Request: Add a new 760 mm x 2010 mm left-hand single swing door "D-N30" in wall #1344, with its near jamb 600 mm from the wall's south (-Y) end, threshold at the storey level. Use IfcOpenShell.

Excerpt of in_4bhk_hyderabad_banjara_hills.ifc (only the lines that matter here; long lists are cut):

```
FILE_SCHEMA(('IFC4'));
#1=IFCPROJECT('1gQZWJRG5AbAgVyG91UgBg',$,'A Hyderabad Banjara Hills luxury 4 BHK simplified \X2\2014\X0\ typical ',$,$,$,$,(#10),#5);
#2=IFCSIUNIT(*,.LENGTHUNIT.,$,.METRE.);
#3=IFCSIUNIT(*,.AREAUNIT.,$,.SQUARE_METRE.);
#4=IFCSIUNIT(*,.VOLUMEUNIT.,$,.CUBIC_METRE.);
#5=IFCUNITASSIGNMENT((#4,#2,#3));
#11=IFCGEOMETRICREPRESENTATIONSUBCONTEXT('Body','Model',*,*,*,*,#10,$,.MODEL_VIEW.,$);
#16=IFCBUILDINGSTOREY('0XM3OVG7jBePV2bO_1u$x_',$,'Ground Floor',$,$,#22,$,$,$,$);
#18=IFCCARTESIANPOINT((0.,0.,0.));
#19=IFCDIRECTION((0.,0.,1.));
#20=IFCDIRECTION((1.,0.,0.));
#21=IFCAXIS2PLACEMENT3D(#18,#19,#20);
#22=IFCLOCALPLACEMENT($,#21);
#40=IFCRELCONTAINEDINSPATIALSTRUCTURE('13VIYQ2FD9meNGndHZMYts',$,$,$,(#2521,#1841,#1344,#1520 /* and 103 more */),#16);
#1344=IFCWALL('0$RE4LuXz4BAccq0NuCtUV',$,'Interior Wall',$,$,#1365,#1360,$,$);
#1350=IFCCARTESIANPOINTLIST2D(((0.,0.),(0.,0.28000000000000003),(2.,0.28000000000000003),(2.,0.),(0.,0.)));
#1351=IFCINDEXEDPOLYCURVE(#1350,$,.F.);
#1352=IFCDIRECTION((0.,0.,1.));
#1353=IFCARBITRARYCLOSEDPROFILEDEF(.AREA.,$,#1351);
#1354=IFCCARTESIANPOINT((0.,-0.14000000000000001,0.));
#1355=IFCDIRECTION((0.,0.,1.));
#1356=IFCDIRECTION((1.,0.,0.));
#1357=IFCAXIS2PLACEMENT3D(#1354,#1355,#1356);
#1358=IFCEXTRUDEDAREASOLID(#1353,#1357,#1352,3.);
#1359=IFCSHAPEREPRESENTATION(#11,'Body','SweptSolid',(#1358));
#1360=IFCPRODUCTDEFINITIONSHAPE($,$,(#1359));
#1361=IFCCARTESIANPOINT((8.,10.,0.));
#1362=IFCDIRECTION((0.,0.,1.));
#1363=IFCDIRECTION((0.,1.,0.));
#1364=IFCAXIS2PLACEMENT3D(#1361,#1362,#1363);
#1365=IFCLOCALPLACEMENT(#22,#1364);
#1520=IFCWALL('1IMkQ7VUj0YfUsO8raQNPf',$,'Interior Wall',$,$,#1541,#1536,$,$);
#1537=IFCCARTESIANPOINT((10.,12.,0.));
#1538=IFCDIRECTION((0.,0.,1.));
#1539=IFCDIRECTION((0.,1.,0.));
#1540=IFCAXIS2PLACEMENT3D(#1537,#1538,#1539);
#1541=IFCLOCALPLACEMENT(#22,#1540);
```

```python
import numpy as np
import ifcopenshell
import ifcopenshell.api.feature
import ifcopenshell.api.geometry
import ifcopenshell.api.root
import ifcopenshell.api.spatial
import ifcopenshell.geom
import ifcopenshell.util.element
import ifcopenshell.util.placement
import ifcopenshell.util.representation
import ifcopenshell.util.shape
import ifcopenshell.util.unit

model = ifcopenshell.open("in_4bhk_hyderabad_banjara_hills.ifc")
unit_scale = ifcopenshell.util.unit.calculate_unit_scale(model)
settings = ifcopenshell.geom.settings()


def volume(element):
    """Net volume in cubic metres, openings subtracted."""
    shape = ifcopenshell.geom.create_shape(settings, element)
    return ifcopenshell.util.shape.get_volume(shape.geometry)


wall = model.by_guid("0$RE4LuXz4BAccq0NuCtUV")
storey = ifcopenshell.util.element.get_container(wall, ifc_class="IfcBuildingStorey")
context = ifcopenshell.util.representation.get_context(model, "Model", "Body", "MODEL_VIEW")
before = volume(wall)

width, height, from_end, sill = 0.76, 2.01, 0.6, 0.0  # metres

# The wall runs along its own X axis, and the end named is its -X end.
wall_shape = ifcopenshell.geom.create_shape(settings, wall)
x, y, z = ifcopenshell.util.shape.get_vertices(wall_shape.geometry).T
start = x.min() + from_end
face, thickness = float(y.min()), float(y.max() - y.min())
wall_matrix = ifcopenshell.util.placement.get_local_placement(wall.ObjectPlacement)
level = ifcopenshell.util.placement.get_local_placement(storey.ObjectPlacement)[2, 3]


def in_wall(x, y):
    """Placement at x, y metres in the wall's axes, at sill height."""
    matrix = wall_matrix.copy()
    matrix[:, 3] = wall_matrix @ np.array([x / unit_scale, y / unit_scale, 0.0, 1.0])
    matrix[2, 3] = level + sill / unit_scale
    return matrix


# Opening: a box that overshoots both wall faces by 50 mm.
opening = ifcopenshell.api.root.create_entity(model, ifc_class="IfcOpeningElement", predefined_type="OPENING")
box = ifcopenshell.api.geometry.add_wall_representation(
    model, context=context, length=width, height=height, thickness=thickness + 0.1
)
ifcopenshell.api.geometry.assign_representation(model, product=opening, representation=box)
ifcopenshell.api.geometry.edit_object_placement(model, product=opening, matrix=in_wall(start, face - 0.05), is_si=False)
ifcopenshell.api.feature.add_feature(model, feature=opening, element=wall)

door = ifcopenshell.api.root.create_entity(model, ifc_class="IfcDoor", name="D-N30", predefined_type="DOOR")
door.OverallWidth, door.OverallHeight = width / unit_scale, height / unit_scale
door.OperationType = "SINGLE_SWING_LEFT"
body = ifcopenshell.api.geometry.add_door_representation(
    model,
    context=context,
    overall_width=door.OverallWidth,
    overall_height=door.OverallHeight,
    operation_type="SINGLE_SWING_LEFT",
    lining_properties={"LiningDepth": thickness / unit_scale, "ThresholdDepth": thickness / unit_scale},
)
ifcopenshell.api.geometry.assign_representation(model, product=door, representation=body)
ifcopenshell.api.spatial.assign_container(model, products=[door], relating_structure=storey)
ifcopenshell.api.feature.add_filling(model, opening=opening, element=door)

# The lining spans the wall, so the door starts at the wall face.
ifcopenshell.api.geometry.edit_object_placement(model, product=door, matrix=in_wall(start, face), is_si=False)

after = volume(wall)

print(f"wall volume {before:.3f} -> {after:.3f} m3")

model.write("in_4bhk_hyderabad_banjara_hills_v2.ifc")
```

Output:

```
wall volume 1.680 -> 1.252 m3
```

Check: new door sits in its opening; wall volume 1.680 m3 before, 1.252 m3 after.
